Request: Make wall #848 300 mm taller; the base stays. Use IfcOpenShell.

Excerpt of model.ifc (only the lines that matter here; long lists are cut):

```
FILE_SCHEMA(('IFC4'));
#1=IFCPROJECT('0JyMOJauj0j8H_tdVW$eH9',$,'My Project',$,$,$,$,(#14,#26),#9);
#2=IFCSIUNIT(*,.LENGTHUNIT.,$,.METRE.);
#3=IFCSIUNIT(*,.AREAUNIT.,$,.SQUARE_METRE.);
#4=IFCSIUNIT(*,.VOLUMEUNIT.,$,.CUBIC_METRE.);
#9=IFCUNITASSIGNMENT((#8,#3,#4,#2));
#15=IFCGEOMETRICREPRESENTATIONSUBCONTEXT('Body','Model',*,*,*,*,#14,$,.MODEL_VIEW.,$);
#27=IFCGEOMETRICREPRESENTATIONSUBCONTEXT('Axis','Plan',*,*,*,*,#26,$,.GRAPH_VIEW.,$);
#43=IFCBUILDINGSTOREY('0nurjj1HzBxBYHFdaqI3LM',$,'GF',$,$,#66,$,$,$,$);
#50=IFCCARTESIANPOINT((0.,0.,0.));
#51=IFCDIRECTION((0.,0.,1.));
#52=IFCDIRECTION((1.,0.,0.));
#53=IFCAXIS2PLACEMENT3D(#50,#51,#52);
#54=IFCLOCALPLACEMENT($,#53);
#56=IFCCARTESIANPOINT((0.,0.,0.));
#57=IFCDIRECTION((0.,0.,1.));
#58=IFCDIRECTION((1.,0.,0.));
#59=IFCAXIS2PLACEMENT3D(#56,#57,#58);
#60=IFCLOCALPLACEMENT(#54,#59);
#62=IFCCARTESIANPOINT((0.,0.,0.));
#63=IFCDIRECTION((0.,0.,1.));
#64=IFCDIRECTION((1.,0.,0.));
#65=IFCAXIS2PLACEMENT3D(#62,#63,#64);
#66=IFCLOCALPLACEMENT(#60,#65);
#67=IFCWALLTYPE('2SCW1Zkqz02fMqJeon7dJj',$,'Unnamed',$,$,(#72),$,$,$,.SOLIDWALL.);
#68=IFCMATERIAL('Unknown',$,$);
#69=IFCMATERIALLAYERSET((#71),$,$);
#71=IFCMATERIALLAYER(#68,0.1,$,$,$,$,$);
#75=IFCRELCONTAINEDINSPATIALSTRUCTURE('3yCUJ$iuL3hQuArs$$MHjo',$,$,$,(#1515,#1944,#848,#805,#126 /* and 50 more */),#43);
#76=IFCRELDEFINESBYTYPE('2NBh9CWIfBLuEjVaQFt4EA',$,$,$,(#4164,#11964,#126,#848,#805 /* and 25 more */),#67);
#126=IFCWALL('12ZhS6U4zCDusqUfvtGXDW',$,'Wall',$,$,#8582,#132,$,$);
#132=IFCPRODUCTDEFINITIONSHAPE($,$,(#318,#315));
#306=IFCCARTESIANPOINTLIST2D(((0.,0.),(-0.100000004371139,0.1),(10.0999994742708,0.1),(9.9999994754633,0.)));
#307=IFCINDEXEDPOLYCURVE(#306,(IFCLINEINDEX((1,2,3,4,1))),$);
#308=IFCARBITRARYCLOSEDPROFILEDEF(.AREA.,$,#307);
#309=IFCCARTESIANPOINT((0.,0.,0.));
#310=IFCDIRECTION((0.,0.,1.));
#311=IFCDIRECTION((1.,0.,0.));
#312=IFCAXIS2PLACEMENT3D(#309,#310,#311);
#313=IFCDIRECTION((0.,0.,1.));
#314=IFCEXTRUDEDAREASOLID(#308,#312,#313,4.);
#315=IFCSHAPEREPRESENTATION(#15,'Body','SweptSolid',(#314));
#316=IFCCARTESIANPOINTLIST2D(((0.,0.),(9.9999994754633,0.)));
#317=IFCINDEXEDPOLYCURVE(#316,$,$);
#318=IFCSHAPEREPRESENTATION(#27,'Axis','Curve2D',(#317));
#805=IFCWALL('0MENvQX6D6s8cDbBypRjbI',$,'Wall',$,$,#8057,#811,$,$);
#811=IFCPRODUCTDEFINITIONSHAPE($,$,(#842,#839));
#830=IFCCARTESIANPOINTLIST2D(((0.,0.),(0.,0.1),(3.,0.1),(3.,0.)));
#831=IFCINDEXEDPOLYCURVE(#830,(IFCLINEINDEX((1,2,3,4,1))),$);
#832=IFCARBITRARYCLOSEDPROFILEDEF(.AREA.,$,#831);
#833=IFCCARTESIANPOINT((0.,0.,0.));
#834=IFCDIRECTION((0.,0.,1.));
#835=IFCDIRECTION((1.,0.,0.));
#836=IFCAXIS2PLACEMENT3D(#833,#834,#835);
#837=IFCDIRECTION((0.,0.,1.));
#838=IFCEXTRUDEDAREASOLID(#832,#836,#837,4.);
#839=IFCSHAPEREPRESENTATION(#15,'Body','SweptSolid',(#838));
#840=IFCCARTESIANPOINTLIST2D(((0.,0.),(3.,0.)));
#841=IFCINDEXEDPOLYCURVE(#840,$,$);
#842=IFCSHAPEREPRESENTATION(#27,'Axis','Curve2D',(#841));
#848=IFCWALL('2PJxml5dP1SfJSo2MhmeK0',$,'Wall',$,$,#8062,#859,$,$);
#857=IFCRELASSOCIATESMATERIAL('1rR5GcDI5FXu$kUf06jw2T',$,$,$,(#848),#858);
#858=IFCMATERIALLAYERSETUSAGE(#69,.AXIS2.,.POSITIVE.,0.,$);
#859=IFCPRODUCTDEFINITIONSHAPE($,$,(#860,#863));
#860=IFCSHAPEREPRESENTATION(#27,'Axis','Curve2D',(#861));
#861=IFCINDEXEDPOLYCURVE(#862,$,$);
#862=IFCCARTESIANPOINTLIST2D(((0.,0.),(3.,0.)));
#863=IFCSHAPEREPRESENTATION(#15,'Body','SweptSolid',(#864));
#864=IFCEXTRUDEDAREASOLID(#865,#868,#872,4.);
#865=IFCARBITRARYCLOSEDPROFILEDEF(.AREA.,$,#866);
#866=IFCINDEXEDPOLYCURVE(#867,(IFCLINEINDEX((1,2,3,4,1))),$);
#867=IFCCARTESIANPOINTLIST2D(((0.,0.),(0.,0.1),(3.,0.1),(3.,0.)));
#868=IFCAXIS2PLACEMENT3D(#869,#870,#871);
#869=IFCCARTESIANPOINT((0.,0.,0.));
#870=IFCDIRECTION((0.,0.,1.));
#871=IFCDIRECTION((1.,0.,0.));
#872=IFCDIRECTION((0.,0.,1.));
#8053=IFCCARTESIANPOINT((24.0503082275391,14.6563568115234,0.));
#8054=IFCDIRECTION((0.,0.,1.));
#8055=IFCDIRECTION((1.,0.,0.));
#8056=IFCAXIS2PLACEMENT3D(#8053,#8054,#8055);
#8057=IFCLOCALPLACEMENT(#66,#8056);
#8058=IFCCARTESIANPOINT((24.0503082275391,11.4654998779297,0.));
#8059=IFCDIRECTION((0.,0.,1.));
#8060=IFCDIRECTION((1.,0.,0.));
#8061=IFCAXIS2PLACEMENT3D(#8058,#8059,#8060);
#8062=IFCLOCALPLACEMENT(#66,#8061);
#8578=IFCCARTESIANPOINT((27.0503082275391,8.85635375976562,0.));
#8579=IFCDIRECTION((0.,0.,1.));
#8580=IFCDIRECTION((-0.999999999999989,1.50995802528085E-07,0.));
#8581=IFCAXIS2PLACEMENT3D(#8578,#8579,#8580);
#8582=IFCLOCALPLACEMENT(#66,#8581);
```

```python
import ifcopenshell
import ifcopenshell.geom
import ifcopenshell.util.representation
import ifcopenshell.util.shape
import ifcopenshell.util.unit

model = ifcopenshell.open("model.ifc")
unit_scale = ifcopenshell.util.unit.calculate_unit_scale(model)
settings = ifcopenshell.geom.settings()


def volume(element):
    """Net volume in cubic metres, openings subtracted."""
    shape = ifcopenshell.geom.create_shape(settings, element)
    return ifcopenshell.util.shape.get_volume(shape.geometry)


wall = model.by_guid("2PJxml5dP1SfJSo2MhmeK0")
before = volume(wall)

body = ifcopenshell.util.representation.get_representation(wall, "Model", "Body")
solid = body.Items[0]
old_height = solid.Depth
solid.Depth += 0.3 / unit_scale
after = volume(wall)

print(f"height {old_height:g} -> {solid.Depth:g}, volume {before:.3f} -> {after:.3f} m3")

model.write("model_updated.ifc")
```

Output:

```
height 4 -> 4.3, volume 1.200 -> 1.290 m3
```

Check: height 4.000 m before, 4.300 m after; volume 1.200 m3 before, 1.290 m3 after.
